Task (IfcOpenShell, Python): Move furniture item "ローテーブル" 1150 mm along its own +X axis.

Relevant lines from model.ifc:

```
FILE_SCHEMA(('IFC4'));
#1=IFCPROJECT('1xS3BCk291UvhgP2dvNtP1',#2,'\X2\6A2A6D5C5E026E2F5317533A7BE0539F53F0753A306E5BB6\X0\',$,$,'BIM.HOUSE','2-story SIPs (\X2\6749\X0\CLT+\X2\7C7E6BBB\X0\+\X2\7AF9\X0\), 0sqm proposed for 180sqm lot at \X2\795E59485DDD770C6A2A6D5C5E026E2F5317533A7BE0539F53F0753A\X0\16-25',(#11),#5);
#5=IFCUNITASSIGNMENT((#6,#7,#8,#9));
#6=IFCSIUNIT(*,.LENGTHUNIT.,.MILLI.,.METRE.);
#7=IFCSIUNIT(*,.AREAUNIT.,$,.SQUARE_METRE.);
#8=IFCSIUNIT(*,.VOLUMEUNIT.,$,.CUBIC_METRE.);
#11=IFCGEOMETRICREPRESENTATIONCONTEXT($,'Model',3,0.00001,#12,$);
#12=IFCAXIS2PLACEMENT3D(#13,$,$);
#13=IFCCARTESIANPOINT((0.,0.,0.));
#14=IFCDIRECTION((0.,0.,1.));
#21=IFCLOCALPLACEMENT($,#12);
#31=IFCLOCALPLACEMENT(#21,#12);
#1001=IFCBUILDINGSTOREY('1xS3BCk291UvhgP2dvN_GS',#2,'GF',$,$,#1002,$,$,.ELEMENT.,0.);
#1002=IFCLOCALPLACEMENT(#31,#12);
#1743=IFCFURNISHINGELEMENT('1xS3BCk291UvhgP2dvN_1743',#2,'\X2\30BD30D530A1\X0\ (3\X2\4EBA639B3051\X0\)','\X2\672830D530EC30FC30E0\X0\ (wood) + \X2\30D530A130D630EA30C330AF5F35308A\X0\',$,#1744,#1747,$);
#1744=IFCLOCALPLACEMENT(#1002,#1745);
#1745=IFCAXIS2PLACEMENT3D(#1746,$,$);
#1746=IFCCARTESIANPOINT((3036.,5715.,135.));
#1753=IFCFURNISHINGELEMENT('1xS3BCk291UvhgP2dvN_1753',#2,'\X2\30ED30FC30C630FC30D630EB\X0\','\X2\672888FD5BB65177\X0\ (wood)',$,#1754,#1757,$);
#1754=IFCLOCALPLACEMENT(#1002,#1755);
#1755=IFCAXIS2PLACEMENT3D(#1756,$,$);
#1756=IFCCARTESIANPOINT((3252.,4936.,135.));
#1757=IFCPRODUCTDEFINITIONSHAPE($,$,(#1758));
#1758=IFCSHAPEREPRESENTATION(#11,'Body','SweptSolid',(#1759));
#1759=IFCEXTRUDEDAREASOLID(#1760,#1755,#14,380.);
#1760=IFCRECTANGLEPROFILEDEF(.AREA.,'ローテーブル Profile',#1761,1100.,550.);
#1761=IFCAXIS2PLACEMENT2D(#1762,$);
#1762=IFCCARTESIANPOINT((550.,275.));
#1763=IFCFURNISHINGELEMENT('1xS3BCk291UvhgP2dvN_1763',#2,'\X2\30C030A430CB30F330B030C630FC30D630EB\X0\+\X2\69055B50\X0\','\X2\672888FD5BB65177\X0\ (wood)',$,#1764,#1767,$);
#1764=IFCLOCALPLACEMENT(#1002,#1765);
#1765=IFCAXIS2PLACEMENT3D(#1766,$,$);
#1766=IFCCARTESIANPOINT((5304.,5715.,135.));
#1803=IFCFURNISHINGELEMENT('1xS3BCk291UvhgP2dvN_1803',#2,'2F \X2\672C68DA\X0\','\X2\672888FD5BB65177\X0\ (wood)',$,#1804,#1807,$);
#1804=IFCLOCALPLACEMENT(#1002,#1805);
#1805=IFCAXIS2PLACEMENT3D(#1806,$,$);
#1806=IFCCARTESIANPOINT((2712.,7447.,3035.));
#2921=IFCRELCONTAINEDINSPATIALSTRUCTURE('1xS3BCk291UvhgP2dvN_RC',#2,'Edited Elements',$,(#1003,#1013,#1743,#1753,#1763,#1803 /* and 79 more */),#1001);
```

```python
import ifcopenshell
import ifcopenshell.api.geometry
import ifcopenshell.util.placement
import ifcopenshell.util.unit

model = ifcopenshell.open("model.ifc")
unit_scale = ifcopenshell.util.unit.calculate_unit_scale(model)

item = model.by_guid("1xS3BCk291UvhgP2dvN_1753")
matrix = ifcopenshell.util.placement.get_local_placement(item.ObjectPlacement)
matrix[:3, 3] += matrix[:3, 0] * 1.15 / unit_scale
ifcopenshell.api.geometry.edit_object_placement(model, product=item, matrix=matrix, is_si=False)

print(ifcopenshell.util.placement.get_local_placement(item.ObjectPlacement).round(3) + 0.0)

model.write("model_edited.ifc")
```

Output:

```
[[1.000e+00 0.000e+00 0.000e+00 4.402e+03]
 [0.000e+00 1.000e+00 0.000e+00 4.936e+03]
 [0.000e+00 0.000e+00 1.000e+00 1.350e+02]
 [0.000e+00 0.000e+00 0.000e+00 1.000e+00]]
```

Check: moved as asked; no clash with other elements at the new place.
